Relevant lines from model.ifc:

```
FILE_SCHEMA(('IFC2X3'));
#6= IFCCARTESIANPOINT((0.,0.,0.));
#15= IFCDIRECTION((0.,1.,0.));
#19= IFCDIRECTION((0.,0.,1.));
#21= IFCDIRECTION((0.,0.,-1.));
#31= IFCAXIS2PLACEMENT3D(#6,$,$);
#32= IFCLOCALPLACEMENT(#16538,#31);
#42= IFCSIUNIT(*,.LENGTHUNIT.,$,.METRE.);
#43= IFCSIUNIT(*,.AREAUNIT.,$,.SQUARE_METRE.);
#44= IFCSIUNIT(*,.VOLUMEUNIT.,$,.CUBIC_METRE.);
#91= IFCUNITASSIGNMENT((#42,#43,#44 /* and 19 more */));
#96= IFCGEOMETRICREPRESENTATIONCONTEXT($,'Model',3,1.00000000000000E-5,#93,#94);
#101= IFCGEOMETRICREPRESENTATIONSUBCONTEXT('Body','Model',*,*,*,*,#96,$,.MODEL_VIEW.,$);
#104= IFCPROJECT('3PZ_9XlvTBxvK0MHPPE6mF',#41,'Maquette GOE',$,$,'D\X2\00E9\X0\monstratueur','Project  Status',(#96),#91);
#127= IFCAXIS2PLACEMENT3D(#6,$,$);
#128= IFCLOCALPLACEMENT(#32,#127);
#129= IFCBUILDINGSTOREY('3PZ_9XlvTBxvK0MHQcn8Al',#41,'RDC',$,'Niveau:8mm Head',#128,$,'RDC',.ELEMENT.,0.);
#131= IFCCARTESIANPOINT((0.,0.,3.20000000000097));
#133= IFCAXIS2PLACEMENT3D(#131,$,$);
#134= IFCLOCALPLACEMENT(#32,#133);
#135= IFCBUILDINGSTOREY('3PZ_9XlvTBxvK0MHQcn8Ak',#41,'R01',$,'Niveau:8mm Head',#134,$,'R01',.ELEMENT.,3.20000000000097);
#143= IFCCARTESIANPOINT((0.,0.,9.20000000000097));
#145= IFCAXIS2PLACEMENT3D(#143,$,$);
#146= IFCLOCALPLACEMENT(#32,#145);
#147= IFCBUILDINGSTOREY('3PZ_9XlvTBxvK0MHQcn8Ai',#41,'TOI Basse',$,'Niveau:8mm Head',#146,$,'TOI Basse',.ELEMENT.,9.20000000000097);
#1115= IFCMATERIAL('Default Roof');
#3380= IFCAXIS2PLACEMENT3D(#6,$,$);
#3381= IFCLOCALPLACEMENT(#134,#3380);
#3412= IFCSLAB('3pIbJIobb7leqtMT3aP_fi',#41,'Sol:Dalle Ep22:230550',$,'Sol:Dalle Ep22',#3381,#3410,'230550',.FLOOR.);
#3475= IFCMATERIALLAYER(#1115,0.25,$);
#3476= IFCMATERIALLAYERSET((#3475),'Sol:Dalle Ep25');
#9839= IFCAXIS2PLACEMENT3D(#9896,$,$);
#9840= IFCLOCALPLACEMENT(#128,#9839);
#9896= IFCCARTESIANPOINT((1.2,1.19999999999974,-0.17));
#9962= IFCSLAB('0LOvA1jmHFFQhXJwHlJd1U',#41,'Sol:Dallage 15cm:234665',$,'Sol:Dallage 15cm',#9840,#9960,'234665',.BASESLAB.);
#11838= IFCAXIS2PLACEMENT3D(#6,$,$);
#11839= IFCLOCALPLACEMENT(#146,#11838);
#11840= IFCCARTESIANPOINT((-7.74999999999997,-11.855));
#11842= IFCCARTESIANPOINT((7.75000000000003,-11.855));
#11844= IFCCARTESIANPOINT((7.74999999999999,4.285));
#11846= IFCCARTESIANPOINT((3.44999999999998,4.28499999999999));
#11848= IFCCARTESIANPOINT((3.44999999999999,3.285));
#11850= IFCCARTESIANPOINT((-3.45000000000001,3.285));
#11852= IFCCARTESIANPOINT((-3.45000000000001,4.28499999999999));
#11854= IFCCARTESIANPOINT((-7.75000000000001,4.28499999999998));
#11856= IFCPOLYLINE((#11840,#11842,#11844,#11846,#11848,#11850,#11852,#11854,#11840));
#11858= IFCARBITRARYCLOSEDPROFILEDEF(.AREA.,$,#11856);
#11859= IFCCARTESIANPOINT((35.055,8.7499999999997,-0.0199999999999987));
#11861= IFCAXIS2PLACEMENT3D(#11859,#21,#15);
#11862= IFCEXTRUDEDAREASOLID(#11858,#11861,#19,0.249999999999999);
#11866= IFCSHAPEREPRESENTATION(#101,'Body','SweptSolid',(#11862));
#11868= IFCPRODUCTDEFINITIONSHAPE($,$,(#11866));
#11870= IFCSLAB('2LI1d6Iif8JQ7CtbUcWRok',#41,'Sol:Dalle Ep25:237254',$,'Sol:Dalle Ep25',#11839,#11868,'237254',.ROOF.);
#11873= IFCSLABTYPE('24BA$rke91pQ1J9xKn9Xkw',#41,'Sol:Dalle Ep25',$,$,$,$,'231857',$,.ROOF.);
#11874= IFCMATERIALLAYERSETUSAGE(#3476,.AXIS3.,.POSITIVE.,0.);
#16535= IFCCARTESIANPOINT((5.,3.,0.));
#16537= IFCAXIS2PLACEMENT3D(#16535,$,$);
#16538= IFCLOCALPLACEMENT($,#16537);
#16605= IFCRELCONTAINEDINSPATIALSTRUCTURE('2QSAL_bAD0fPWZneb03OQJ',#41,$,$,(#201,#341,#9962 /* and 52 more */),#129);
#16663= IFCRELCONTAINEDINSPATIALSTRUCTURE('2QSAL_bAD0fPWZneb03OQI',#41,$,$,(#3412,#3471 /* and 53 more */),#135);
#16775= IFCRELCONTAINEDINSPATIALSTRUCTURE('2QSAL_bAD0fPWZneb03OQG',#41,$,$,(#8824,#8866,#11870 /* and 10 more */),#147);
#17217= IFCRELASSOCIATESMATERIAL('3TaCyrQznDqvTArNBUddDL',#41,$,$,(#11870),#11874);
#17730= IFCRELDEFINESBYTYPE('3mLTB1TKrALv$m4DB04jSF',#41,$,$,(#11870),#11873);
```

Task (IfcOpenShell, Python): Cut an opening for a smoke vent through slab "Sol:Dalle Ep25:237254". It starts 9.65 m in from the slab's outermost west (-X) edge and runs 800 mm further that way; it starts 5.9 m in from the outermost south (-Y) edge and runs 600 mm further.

```python
import numpy as np
import ifcopenshell
import ifcopenshell.api.feature
import ifcopenshell.api.geometry
import ifcopenshell.api.root
import ifcopenshell.geom
import ifcopenshell.util.placement
import ifcopenshell.util.representation
import ifcopenshell.util.shape
import ifcopenshell.util.unit

model = ifcopenshell.open("model.ifc")
unit_scale = ifcopenshell.util.unit.calculate_unit_scale(model)
settings = ifcopenshell.geom.settings()


def volume(element):
    """Net volume in cubic metres, openings subtracted."""
    shape = ifcopenshell.geom.create_shape(settings, element)
    return ifcopenshell.util.shape.get_volume(shape.geometry)


slab = model.by_guid("2LI1d6Iif8JQ7CtbUcWRok")
before = volume(slab)

# Extent in the slab's own axes, in metres. The edges named are its -X and -Y sides.
slab_shape = ifcopenshell.geom.create_shape(settings, slab)
vertices = ifcopenshell.util.shape.get_vertices(slab_shape.geometry)
x_min, y_min, bottom = vertices.min(axis=0)
top = vertices[:, 2].max()

opening = ifcopenshell.api.root.create_entity(model, ifc_class="IfcOpeningElement", name="Smoke vent opening")
context = ifcopenshell.util.representation.get_context(model, "Model", "Body", "MODEL_VIEW")
width, depth = 0.8, 0.6
outline = [(0.0, 0.0), (width, 0.0), (width, depth), (0.0, depth), (0.0, 0.0)]
# Overshoot both faces by 50 mm so the cut is clean.
shape = ifcopenshell.api.geometry.add_slab_representation(
    model, context=context, depth=top - bottom + 0.1, polyline=outline
)
ifcopenshell.api.geometry.assign_representation(model, product=opening, representation=shape)

matrix = ifcopenshell.util.placement.get_local_placement(slab.ObjectPlacement)
matrix[:, 3] = matrix @ np.append(np.array([x_min + 9.65, y_min + 5.9, bottom - 0.05]) / unit_scale, 1.0)
ifcopenshell.api.geometry.edit_object_placement(model, product=opening, matrix=matrix, is_si=False)
ifcopenshell.api.feature.add_feature(model, feature=opening, element=slab)

after = volume(slab)

print(f"slab volume {before:.3f} -> {after:.3f} m3")

model.write("model_rev.ifc")
```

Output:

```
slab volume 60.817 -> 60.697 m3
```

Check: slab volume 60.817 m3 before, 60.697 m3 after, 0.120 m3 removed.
